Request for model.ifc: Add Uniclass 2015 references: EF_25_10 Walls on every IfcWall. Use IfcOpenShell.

First a look at what the model holds.

```python
import ifcopenshell

model = ifcopenshell.open("model.ifc")
print(model.schema)
print("classifications:", [c.Name for c in model.by_type("IfcClassification")])
for ifc_class in ("IfcDoor", "IfcRoof", "IfcStair", "IfcWall", "IfcWindow"):
    print(ifc_class, len(model.by_type(ifc_class)))
```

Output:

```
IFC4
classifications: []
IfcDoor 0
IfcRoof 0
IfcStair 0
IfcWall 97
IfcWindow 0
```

```python
import ifcopenshell
import ifcopenshell.api.classification

model = ifcopenshell.open("model.ifc")

system = ifcopenshell.api.classification.add_classification(model, classification="Uniclass 2015")

codes = {
    "IfcWall": ("EF_25_10", "Walls"),
}
for ifc_class, (code, name) in codes.items():
    products = model.by_type(ifc_class)
    ifcopenshell.api.classification.add_reference(
        model, products=products, classification=system, identification=code, name=name
    )
    print(code, len(products))

model.write("model_edited.ifc")
```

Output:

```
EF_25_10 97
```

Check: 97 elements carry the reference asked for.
